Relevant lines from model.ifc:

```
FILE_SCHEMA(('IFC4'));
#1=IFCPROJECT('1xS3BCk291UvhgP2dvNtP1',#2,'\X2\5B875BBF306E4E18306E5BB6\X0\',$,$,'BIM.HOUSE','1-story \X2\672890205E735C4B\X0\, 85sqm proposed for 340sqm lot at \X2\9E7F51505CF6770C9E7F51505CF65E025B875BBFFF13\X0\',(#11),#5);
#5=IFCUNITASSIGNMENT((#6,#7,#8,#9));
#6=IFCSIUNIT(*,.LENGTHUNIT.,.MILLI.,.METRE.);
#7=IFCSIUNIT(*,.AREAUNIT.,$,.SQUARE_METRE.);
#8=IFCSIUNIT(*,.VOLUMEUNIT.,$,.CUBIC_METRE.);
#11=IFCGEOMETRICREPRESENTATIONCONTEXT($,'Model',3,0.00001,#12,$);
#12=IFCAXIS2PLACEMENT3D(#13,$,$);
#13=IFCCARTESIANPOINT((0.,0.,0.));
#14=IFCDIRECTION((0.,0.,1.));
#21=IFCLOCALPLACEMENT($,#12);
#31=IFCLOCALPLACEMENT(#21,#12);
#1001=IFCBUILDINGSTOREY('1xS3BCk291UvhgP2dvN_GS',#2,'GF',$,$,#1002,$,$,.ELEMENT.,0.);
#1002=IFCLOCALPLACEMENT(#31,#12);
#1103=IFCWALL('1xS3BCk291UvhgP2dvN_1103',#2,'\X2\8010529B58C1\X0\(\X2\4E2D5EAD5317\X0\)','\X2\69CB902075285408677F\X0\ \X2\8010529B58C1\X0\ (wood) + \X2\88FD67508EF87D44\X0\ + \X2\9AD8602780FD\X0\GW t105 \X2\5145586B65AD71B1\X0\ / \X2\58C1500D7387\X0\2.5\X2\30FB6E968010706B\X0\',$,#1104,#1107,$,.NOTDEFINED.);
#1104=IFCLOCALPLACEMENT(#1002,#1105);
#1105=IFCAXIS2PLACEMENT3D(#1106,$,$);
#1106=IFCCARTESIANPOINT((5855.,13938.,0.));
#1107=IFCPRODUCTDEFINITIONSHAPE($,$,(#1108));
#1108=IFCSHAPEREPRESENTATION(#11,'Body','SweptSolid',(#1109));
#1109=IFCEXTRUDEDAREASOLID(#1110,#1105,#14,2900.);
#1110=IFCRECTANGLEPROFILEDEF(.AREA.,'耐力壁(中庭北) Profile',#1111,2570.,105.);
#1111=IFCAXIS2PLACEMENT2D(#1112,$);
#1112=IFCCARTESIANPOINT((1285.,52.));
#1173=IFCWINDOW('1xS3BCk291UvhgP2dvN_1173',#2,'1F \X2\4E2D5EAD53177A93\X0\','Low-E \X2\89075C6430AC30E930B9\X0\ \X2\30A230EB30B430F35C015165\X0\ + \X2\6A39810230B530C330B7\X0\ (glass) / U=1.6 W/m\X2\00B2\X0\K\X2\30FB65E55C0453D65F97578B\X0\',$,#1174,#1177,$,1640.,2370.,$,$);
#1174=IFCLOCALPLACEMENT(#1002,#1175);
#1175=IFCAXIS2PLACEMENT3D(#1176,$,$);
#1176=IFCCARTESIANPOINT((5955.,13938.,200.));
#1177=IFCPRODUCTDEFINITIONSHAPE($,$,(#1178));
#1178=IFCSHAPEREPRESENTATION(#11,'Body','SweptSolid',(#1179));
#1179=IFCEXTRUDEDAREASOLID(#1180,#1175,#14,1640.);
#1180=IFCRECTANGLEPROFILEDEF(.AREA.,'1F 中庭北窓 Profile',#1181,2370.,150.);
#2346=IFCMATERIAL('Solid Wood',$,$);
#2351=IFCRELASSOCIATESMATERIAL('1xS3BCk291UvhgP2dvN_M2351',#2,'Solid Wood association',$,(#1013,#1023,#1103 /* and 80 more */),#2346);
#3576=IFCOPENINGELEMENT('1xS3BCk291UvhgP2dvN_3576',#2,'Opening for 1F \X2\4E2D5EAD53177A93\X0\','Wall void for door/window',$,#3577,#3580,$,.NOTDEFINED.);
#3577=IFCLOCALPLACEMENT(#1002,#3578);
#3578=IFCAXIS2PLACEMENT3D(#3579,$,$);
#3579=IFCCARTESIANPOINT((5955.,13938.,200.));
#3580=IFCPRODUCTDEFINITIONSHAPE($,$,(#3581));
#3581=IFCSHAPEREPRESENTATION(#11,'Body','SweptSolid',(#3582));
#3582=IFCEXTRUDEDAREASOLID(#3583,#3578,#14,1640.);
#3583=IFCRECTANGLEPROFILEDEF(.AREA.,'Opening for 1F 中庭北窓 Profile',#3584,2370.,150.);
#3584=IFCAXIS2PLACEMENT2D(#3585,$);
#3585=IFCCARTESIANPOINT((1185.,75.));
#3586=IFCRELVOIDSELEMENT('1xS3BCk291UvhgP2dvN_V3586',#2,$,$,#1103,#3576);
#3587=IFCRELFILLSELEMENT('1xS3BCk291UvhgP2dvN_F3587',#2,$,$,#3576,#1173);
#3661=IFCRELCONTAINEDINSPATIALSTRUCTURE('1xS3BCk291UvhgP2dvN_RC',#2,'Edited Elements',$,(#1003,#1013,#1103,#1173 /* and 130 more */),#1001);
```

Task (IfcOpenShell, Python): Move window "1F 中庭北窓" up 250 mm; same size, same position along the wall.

```python
import numpy as np
import ifcopenshell
import ifcopenshell.api.geometry
import ifcopenshell.util.placement
import ifcopenshell.util.unit

model = ifcopenshell.open("model.ifc")
unit_scale = ifcopenshell.util.unit.calculate_unit_scale(model)

window = model.by_guid("1xS3BCk291UvhgP2dvN_1173")
opening = window.FillsVoids[0].RelatingOpeningElement
dz = 250.0

shift = np.array([0.0, 0.0, dz])
# The window is not placed relative to its opening, so move both.
for product in (opening, window):
    matrix = ifcopenshell.util.placement.get_local_placement(product.ObjectPlacement)
    matrix[:3, 3] += shift
    ifcopenshell.api.geometry.edit_object_placement(model, product=product, matrix=matrix, is_si=False)

print(f"moved by {dz * unit_scale:+.3f} m")

model.write("model_rev.ifc")
```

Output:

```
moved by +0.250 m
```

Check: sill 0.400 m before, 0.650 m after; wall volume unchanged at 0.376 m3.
